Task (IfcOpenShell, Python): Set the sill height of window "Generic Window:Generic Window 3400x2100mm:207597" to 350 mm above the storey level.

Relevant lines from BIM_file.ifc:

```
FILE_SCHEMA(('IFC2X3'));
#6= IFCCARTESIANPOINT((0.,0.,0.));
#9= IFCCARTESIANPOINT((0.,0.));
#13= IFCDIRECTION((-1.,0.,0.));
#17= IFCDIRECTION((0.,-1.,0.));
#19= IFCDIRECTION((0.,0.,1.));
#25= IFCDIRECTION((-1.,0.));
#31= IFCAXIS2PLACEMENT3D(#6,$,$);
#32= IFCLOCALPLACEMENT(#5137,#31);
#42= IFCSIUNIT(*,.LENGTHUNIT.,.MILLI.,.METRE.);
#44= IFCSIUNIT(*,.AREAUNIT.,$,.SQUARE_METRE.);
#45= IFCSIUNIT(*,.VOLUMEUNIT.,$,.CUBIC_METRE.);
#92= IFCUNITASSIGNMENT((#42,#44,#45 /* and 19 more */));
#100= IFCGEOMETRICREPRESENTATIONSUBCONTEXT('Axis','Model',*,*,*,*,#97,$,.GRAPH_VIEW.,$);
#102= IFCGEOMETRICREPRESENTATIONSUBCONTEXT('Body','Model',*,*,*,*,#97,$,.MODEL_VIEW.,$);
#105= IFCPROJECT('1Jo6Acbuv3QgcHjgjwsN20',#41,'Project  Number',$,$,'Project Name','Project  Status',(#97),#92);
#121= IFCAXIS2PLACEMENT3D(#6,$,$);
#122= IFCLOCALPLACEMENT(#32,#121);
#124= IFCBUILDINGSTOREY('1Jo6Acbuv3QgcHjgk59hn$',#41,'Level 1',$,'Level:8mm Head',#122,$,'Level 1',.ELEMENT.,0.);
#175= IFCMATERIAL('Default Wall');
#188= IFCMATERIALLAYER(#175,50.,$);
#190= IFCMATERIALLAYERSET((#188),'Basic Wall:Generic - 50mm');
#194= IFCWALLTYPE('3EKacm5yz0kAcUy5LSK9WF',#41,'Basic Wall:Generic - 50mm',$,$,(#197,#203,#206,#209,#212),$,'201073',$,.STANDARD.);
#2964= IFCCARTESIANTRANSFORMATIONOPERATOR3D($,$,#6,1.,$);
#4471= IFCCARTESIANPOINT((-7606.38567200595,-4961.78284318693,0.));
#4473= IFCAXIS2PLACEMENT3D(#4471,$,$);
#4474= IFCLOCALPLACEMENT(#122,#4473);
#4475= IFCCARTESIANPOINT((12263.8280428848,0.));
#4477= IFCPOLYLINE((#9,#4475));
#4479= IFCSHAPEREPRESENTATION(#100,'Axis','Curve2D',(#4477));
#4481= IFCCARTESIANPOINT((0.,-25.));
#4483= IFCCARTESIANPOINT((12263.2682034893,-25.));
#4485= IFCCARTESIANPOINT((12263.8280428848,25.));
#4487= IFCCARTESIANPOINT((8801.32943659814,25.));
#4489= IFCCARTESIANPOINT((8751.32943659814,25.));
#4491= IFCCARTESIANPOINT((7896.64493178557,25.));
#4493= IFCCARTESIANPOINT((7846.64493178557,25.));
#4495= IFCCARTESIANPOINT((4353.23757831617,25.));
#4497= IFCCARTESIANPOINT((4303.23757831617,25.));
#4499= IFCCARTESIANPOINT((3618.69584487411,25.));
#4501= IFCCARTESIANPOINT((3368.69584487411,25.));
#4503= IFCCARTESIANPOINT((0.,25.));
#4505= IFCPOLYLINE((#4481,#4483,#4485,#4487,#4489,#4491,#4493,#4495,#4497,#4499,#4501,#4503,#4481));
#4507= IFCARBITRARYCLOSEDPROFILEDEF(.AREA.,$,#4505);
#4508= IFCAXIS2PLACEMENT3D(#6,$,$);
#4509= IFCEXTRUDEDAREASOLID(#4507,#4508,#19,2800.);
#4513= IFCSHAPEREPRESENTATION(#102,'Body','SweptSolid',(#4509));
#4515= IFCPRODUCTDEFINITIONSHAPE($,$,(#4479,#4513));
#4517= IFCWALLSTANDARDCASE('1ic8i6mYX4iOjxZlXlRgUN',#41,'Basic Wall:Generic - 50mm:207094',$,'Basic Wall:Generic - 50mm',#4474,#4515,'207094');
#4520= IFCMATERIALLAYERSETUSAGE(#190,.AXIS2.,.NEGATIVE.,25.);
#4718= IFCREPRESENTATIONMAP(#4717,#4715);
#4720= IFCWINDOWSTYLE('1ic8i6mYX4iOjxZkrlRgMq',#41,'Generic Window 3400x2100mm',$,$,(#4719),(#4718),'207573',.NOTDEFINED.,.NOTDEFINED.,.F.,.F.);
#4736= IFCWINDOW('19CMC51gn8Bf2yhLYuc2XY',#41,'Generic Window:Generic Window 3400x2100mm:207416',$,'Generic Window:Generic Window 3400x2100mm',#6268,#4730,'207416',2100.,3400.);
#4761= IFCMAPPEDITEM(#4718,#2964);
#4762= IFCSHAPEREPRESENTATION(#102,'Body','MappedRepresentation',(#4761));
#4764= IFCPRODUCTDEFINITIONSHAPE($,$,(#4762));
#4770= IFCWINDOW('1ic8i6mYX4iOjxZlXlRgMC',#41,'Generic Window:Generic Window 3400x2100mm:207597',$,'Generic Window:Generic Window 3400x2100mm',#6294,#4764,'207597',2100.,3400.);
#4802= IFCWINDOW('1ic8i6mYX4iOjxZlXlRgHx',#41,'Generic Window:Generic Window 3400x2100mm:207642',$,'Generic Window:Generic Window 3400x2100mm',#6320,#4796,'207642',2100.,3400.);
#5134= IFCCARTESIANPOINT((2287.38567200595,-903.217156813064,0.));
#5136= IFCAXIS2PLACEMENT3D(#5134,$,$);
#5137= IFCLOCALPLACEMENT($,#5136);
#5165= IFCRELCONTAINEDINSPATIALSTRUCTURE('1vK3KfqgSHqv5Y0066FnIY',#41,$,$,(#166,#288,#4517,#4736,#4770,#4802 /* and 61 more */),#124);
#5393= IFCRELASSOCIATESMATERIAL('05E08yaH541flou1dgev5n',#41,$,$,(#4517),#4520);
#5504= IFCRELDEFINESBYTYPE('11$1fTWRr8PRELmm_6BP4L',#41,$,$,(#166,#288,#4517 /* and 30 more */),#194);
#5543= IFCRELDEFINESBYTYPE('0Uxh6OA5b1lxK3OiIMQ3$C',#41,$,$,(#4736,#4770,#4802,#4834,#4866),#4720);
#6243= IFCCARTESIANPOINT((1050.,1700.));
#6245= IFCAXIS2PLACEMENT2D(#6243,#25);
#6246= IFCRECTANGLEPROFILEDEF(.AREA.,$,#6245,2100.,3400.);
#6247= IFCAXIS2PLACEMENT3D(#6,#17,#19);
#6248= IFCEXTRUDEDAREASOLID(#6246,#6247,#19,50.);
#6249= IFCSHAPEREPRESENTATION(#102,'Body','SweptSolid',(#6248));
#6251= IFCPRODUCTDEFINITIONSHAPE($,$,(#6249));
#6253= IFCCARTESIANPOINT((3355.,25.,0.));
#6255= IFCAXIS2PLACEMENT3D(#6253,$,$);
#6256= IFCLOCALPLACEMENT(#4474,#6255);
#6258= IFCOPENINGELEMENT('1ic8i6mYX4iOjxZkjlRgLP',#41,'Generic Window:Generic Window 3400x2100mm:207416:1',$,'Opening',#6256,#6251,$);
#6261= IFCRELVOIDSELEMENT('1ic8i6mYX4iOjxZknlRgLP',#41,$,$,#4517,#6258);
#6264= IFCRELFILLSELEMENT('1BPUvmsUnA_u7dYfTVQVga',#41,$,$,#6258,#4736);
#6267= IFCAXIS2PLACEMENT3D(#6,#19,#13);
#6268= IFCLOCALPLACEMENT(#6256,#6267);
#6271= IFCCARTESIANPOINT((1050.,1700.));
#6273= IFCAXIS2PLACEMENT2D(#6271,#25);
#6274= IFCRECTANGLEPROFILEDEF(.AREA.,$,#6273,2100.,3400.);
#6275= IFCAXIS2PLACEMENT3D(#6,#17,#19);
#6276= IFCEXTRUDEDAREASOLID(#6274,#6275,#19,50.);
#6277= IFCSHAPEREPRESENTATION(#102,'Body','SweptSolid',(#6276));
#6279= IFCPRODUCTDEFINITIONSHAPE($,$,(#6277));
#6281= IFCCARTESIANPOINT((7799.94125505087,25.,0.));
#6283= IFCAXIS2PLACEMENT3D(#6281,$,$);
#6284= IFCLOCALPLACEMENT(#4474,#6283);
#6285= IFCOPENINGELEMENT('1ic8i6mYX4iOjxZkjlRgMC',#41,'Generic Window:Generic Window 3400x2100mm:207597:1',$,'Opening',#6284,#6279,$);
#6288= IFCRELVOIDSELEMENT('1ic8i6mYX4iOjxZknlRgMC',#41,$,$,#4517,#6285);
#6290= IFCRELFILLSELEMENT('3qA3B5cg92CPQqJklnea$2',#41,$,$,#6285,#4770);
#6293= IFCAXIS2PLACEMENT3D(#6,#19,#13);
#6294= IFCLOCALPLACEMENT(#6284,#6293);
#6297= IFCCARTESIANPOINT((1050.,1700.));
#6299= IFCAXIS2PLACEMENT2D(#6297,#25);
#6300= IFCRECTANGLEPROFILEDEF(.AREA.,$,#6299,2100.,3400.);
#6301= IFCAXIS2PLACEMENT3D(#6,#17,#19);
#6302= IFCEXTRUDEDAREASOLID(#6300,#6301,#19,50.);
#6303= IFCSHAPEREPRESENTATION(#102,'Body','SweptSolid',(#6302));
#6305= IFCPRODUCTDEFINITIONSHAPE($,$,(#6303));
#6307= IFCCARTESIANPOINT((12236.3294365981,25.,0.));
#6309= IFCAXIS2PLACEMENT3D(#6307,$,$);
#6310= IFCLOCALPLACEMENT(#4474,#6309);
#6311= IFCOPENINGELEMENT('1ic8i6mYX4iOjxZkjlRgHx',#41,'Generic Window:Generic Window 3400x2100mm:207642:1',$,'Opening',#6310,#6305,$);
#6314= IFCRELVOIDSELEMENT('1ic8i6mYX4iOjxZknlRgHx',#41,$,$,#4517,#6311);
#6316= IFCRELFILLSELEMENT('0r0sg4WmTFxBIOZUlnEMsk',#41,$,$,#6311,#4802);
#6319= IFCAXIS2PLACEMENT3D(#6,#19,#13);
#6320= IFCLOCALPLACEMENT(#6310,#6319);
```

```python
import numpy as np
import ifcopenshell
import ifcopenshell.api.geometry
import ifcopenshell.geom
import ifcopenshell.util.element
import ifcopenshell.util.placement
import ifcopenshell.util.shape
import ifcopenshell.util.unit

model = ifcopenshell.open("BIM_file.ifc")
unit_scale = ifcopenshell.util.unit.calculate_unit_scale(model)

window = model.by_id(4770)
opening = window.FillsVoids[0].RelatingOpeningElement
storey = ifcopenshell.util.element.get_container(window, ifc_class="IfcBuildingStorey")
level = ifcopenshell.util.placement.get_local_placement(storey.ObjectPlacement)[2, 3]

# The opening's origin need not be at the sill, so measure its lowest point.
shape = ifcopenshell.geom.create_shape(ifcopenshell.geom.settings(), opening)
bottom = ifcopenshell.util.shape.get_shape_bottom_elevation(shape, shape.geometry) / unit_scale
dz = level + 0.35 / unit_scale - bottom

shift = np.array([0.0, 0.0, dz])
# The window is placed relative to its opening, so it follows when the opening moves.
matrix = ifcopenshell.util.placement.get_local_placement(opening.ObjectPlacement)
matrix[:3, 3] += shift
ifcopenshell.api.geometry.edit_object_placement(
    model, product=opening, matrix=matrix, is_si=False, should_transform_children=True
)

print(f"moved by {dz * unit_scale:+.3f} m")

model.write("BIM_file_edited.ifc")
```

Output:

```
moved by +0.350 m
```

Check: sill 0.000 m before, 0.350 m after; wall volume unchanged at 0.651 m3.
